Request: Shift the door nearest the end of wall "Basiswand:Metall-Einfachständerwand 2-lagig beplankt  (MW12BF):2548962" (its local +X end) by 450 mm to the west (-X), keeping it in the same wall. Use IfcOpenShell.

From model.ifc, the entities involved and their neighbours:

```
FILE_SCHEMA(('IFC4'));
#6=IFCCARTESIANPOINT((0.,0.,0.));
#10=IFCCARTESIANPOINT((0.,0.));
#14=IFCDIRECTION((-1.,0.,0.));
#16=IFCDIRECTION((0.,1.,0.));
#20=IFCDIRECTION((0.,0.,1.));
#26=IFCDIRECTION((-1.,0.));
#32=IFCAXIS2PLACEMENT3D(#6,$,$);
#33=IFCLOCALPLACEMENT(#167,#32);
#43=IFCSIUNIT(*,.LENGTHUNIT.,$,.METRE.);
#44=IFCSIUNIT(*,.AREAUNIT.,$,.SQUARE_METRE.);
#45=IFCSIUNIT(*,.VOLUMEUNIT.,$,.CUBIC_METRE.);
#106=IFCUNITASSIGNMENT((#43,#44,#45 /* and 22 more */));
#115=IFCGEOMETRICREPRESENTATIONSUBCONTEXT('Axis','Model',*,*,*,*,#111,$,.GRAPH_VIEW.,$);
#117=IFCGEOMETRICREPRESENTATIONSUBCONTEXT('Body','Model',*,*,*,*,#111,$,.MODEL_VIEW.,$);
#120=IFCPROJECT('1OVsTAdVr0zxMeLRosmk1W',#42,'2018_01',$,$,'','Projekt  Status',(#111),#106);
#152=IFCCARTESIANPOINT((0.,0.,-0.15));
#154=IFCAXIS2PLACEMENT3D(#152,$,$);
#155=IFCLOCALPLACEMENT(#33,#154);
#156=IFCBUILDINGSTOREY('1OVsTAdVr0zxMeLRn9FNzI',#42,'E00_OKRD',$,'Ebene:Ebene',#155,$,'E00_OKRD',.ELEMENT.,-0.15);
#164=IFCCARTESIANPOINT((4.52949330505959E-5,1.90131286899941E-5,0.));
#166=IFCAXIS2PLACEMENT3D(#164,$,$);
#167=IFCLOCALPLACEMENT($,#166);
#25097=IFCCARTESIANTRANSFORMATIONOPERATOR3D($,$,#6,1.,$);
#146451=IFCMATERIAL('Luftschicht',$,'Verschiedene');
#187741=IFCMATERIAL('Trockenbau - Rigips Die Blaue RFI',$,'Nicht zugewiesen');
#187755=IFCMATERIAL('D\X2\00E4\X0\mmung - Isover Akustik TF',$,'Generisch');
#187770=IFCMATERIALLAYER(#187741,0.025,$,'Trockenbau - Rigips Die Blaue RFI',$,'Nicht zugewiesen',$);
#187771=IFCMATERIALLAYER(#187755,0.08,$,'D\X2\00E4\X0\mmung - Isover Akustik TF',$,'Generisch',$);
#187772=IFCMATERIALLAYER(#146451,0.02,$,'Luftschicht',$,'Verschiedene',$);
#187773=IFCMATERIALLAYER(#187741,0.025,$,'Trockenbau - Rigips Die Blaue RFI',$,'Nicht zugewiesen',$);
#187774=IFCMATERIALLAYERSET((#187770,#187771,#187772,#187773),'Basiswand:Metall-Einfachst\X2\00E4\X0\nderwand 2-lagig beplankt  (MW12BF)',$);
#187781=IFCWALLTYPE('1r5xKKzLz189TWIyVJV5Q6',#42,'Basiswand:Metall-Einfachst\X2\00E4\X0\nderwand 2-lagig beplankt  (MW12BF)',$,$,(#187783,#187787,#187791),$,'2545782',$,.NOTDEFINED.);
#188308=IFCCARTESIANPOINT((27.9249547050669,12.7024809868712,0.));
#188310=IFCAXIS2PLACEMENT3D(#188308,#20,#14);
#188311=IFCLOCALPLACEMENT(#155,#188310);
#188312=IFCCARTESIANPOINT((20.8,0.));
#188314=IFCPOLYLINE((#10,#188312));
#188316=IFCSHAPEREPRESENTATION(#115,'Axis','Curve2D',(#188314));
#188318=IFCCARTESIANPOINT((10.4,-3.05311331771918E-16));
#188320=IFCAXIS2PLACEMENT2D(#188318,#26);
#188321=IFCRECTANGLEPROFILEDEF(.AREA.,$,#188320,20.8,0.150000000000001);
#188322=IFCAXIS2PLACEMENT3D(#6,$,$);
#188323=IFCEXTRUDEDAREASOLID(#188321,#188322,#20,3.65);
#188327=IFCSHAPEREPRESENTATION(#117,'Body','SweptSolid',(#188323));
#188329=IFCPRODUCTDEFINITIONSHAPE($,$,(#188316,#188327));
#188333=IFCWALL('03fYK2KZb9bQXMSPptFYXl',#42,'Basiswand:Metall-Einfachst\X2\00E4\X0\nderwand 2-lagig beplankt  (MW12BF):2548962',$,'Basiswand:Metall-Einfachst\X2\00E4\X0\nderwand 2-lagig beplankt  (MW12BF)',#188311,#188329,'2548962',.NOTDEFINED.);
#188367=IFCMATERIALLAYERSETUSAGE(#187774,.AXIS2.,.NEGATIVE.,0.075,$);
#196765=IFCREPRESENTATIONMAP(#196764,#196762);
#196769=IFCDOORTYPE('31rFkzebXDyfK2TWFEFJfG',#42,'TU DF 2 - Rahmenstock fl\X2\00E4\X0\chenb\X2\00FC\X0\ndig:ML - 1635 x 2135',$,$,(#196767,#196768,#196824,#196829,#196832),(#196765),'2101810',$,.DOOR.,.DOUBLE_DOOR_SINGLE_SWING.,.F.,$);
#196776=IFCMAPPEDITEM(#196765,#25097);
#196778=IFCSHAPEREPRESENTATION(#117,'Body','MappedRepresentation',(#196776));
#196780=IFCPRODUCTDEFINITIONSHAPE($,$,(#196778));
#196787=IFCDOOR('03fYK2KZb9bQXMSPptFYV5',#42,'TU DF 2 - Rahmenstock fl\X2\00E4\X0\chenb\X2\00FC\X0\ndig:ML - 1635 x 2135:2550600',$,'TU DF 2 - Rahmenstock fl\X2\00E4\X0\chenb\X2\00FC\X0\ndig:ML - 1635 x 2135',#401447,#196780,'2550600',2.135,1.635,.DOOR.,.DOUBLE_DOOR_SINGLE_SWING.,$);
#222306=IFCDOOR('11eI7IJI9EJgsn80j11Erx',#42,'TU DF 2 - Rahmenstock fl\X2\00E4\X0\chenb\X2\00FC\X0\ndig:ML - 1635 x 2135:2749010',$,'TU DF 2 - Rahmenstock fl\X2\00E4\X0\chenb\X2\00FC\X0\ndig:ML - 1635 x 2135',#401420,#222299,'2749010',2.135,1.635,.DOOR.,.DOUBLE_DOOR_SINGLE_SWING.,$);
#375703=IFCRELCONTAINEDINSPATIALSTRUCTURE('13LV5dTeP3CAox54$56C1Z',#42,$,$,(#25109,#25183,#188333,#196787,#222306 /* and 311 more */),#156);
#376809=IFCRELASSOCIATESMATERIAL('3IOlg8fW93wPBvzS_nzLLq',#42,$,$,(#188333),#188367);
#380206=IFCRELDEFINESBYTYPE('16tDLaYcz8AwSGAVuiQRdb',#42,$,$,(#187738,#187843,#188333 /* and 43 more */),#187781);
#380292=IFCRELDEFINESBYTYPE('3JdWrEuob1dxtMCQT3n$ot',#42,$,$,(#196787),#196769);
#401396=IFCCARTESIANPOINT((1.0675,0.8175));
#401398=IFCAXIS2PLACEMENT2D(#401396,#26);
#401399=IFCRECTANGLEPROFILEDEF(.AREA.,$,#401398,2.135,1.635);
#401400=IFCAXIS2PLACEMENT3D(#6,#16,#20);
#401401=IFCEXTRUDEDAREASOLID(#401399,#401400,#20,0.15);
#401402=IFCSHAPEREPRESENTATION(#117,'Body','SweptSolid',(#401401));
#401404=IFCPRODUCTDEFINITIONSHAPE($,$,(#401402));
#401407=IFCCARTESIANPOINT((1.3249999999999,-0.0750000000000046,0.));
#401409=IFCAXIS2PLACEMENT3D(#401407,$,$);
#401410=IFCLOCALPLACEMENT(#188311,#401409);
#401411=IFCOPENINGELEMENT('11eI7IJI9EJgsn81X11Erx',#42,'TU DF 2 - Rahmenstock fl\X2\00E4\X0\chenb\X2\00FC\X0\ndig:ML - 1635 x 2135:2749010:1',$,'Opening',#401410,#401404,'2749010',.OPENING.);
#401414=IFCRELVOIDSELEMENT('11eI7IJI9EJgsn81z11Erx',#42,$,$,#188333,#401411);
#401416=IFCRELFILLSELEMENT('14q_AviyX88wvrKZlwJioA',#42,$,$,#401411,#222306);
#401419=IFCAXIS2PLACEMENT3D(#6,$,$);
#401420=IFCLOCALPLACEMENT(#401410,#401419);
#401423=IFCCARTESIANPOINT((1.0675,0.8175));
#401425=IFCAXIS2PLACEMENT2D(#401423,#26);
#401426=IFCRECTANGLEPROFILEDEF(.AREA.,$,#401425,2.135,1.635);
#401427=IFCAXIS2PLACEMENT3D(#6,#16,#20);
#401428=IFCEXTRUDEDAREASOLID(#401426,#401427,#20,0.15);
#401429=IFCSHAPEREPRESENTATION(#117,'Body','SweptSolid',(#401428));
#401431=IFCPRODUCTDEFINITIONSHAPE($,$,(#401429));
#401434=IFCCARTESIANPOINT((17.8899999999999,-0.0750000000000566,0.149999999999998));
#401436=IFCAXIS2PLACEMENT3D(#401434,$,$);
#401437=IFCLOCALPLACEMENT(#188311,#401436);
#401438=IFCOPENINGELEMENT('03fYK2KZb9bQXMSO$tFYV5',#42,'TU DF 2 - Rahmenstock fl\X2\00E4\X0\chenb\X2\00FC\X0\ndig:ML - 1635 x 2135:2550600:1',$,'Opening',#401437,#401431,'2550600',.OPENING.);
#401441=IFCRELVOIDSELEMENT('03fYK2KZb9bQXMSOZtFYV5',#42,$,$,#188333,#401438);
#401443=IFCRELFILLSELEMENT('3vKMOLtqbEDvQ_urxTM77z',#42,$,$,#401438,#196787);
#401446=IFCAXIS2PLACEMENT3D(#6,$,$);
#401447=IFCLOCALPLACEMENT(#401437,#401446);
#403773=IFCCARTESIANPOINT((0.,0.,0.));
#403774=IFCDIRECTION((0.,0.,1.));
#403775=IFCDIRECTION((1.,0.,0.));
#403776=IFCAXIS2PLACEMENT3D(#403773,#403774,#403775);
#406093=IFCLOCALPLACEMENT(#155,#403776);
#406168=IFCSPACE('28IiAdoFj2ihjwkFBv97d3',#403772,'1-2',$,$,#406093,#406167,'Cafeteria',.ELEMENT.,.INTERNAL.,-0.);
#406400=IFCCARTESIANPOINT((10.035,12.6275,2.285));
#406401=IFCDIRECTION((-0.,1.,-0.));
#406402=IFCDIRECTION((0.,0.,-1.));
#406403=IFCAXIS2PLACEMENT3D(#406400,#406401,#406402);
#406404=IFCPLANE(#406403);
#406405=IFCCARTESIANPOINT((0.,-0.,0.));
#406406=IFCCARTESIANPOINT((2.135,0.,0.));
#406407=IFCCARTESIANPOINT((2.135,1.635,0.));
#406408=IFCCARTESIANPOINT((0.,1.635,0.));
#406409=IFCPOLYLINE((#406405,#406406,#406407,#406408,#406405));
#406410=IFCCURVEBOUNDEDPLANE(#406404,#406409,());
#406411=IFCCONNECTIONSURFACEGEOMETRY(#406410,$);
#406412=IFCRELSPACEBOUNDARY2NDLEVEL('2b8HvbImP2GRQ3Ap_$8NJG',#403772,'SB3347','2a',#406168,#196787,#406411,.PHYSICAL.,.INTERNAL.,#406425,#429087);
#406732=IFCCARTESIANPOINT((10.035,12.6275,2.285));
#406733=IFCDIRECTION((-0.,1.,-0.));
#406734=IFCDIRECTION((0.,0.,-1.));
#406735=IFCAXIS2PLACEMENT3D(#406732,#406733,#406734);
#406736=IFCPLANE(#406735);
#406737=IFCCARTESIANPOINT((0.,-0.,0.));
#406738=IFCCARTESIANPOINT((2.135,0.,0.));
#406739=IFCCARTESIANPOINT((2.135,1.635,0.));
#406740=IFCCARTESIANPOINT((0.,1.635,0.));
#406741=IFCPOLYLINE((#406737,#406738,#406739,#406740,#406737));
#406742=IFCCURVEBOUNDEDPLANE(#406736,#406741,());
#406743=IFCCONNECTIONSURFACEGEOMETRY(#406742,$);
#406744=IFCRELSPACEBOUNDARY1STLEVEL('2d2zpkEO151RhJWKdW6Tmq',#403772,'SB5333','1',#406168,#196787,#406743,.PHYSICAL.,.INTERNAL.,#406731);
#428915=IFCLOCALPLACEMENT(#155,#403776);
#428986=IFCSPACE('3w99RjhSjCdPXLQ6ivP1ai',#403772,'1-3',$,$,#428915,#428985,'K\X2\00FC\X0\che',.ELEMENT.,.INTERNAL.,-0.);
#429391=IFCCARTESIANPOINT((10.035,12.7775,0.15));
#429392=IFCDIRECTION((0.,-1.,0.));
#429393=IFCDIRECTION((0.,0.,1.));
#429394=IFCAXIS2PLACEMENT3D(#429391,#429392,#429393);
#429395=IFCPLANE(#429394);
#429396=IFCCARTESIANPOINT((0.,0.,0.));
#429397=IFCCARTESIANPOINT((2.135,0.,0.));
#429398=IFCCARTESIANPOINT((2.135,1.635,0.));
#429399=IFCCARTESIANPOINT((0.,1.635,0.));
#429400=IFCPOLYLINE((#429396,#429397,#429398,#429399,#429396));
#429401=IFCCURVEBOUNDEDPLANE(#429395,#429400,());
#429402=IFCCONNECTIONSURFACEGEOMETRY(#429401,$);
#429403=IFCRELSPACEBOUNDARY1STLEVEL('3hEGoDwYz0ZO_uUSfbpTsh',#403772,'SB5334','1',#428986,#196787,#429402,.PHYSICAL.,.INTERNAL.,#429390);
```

```python
import numpy as np
import ifcopenshell
import ifcopenshell.api.geometry
import ifcopenshell.util.placement

model = ifcopenshell.open("model.ifc")

door = model.by_id(196787)
opening = door.FillsVoids[0].RelatingOpeningElement
wall = opening.VoidsElements[0].RelatingBuildingElement

wall_matrix = ifcopenshell.util.placement.get_local_placement(wall.ObjectPlacement)
shift = wall_matrix[:3, 0] * 0.45
before = ifcopenshell.util.placement.get_local_placement(door.ObjectPlacement)[:3, 3].copy()

# The door is placed relative to its opening, so it follows when the opening moves.
matrix = ifcopenshell.util.placement.get_local_placement(opening.ObjectPlacement)
matrix[:3, 3] += shift
ifcopenshell.api.geometry.edit_object_placement(
    model, product=opening, matrix=matrix, is_si=False, should_transform_children=True
)

# Space boundary surfaces are stored in each space's coordinates; move them too.
for rel in door.ProvidesBoundaries:
    if not rel.ConnectionGeometry:
        continue
    surface = rel.ConnectionGeometry.SurfaceOnRelatingElement.BasisSurface
    space_matrix = ifcopenshell.util.placement.get_local_placement(rel.RelatingSpace.ObjectPlacement)
    point = np.array(surface.Position.Location.Coordinates) + space_matrix[:3, :3].T @ shift
    surface.Position = model.createIfcAxis2Placement3D(
        model.createIfcCartesianPoint(point.tolist()), surface.Position.Axis, surface.Position.RefDirection
    )

after = ifcopenshell.util.placement.get_local_placement(door.ObjectPlacement)[:3, 3]
print("door moved by", (after - before).round(3) + 0.0)

model.write("model_updated.ifc")
```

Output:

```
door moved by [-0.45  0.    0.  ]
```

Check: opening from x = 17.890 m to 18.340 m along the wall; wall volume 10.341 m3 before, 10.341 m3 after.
